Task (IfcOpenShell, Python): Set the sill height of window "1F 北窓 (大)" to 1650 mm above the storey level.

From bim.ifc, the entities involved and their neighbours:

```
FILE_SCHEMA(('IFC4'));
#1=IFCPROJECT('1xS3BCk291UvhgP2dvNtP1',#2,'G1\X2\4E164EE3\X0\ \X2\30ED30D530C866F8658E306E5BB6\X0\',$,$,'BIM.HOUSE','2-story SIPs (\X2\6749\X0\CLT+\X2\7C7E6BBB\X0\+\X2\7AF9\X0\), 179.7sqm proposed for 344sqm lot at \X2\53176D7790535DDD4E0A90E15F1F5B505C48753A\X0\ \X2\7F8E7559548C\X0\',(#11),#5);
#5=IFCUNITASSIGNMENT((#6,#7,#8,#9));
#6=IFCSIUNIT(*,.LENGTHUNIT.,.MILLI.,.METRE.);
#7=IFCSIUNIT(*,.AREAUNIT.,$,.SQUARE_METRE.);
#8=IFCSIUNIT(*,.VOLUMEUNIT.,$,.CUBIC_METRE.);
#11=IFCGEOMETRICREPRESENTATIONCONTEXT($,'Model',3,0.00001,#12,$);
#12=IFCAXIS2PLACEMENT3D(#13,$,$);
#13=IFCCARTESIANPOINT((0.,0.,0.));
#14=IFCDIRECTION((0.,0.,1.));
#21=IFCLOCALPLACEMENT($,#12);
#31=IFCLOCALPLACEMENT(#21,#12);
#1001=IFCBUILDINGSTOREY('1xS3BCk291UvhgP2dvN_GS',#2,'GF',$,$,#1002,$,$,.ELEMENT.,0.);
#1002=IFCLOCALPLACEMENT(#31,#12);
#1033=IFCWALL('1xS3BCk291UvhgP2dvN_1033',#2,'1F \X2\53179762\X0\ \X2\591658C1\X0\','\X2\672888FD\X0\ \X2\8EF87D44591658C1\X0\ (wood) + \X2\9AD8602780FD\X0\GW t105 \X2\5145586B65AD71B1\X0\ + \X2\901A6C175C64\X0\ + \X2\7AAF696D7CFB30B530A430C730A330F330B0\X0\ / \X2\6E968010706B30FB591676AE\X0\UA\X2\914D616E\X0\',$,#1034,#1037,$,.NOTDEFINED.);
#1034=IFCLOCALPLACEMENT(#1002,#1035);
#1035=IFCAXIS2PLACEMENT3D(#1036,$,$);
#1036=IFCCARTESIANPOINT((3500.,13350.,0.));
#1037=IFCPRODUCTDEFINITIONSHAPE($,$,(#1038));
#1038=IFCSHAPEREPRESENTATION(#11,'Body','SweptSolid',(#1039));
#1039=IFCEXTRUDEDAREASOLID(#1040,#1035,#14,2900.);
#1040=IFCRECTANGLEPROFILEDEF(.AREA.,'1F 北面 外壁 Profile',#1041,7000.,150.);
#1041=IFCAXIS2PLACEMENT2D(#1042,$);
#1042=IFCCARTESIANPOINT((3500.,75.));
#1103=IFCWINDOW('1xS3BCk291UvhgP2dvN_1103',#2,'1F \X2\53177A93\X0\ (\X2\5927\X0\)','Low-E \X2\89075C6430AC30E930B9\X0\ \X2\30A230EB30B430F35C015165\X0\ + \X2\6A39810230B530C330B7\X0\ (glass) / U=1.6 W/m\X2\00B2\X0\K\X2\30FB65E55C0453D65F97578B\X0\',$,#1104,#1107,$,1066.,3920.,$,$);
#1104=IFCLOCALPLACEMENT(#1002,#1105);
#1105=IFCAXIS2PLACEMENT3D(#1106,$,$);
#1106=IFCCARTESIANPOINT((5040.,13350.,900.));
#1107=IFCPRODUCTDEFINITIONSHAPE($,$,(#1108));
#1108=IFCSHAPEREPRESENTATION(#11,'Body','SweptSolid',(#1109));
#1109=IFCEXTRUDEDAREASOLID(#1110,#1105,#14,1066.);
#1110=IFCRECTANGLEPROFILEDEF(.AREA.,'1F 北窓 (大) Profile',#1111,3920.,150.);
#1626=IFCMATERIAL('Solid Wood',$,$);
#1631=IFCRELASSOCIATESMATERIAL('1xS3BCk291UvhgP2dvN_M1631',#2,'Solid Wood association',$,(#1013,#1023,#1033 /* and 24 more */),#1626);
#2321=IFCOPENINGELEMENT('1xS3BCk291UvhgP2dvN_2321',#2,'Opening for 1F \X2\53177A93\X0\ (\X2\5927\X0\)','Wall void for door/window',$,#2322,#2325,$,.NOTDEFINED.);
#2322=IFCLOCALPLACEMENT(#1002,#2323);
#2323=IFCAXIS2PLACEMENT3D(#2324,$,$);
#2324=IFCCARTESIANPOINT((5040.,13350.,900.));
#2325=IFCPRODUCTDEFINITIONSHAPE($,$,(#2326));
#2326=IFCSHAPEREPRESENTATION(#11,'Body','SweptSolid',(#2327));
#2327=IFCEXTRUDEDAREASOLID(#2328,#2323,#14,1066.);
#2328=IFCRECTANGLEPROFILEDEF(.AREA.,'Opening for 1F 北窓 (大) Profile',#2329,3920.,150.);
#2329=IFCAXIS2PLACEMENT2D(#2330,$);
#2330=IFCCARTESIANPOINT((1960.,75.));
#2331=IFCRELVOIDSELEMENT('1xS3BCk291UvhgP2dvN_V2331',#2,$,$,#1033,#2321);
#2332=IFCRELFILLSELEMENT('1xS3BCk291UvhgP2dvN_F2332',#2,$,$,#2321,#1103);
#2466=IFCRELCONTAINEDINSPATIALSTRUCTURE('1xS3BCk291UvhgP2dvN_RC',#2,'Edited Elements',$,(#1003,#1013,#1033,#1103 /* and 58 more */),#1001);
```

```python
import numpy as np
import ifcopenshell
import ifcopenshell.api.geometry
import ifcopenshell.geom
import ifcopenshell.util.element
import ifcopenshell.util.placement
import ifcopenshell.util.shape
import ifcopenshell.util.unit

model = ifcopenshell.open("bim.ifc")
unit_scale = ifcopenshell.util.unit.calculate_unit_scale(model)

window = model.by_guid("1xS3BCk291UvhgP2dvN_1103")
opening = window.FillsVoids[0].RelatingOpeningElement
storey = ifcopenshell.util.element.get_container(window, ifc_class="IfcBuildingStorey")
level = ifcopenshell.util.placement.get_local_placement(storey.ObjectPlacement)[2, 3]

# The opening's origin need not be at the sill, so measure its lowest point.
shape = ifcopenshell.geom.create_shape(ifcopenshell.geom.settings(), opening)
bottom = ifcopenshell.util.shape.get_shape_bottom_elevation(shape, shape.geometry) / unit_scale
dz = level + 1.65 / unit_scale - bottom

shift = np.array([0.0, 0.0, dz])
# The window is not placed relative to its opening, so move both.
for product in (opening, window):
    matrix = ifcopenshell.util.placement.get_local_placement(product.ObjectPlacement)
    matrix[:3, 3] += shift
    ifcopenshell.api.geometry.edit_object_placement(model, product=product, matrix=matrix, is_si=False)

print(f"moved by {dz * unit_scale:+.3f} m")

model.write("bim_v2.ifc")
```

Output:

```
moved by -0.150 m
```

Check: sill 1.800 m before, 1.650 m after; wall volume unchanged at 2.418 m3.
